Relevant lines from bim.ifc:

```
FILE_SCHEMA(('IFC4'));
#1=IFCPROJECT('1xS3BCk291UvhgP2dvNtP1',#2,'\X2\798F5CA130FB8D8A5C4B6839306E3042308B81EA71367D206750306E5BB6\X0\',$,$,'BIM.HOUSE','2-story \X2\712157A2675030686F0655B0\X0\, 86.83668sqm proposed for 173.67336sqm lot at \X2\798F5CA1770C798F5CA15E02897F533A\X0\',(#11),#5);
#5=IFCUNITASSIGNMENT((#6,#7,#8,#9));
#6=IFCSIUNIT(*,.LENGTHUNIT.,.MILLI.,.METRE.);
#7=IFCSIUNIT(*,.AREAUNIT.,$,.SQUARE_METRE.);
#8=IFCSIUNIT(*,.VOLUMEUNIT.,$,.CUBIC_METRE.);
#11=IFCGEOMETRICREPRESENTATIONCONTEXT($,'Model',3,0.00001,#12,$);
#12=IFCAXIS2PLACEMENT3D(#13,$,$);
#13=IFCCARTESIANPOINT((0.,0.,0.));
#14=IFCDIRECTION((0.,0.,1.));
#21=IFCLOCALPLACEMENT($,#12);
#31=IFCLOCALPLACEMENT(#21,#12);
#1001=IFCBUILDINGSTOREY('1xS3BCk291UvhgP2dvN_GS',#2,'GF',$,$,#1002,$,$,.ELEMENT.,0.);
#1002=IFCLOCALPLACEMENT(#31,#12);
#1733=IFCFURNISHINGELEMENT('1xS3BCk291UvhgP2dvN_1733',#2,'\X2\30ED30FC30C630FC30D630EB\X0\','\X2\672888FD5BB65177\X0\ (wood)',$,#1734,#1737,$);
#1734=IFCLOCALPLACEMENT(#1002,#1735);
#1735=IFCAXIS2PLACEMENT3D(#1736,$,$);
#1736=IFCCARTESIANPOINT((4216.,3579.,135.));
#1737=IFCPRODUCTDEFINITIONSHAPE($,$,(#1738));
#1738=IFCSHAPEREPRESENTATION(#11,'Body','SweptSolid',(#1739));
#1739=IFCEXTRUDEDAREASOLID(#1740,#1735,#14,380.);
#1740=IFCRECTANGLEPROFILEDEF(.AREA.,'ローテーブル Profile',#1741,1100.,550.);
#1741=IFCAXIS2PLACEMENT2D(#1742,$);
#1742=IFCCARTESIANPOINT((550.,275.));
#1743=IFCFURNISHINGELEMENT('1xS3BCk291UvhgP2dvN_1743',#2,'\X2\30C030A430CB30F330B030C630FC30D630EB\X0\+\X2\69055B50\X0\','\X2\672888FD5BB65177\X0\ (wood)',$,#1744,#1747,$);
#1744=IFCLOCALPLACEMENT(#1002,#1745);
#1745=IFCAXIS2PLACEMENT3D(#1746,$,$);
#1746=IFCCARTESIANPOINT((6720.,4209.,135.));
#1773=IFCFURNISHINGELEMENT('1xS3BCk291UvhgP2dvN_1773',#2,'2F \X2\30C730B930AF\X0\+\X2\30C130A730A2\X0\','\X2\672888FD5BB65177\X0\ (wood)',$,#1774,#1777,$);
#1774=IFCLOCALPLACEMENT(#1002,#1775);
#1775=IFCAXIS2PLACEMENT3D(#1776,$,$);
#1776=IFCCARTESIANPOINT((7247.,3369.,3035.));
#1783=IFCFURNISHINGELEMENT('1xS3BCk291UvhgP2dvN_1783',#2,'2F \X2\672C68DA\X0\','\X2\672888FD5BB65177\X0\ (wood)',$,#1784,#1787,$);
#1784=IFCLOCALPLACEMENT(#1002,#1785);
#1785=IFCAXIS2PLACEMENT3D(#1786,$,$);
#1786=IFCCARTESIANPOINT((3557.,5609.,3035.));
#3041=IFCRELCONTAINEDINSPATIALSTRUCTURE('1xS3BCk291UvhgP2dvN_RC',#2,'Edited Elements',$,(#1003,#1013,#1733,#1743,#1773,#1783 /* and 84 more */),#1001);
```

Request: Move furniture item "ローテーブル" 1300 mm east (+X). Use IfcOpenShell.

```python
import ifcopenshell
import ifcopenshell.api.geometry
import ifcopenshell.util.placement
import ifcopenshell.util.unit

model = ifcopenshell.open("bim.ifc")
unit_scale = ifcopenshell.util.unit.calculate_unit_scale(model)

item = model.by_guid("1xS3BCk291UvhgP2dvN_1733")
matrix = ifcopenshell.util.placement.get_local_placement(item.ObjectPlacement)
matrix[0, 3] += 1.3 / unit_scale
ifcopenshell.api.geometry.edit_object_placement(model, product=item, matrix=matrix, is_si=False)

print(ifcopenshell.util.placement.get_local_placement(item.ObjectPlacement).round(3) + 0.0)

model.write("bim_v2.ifc")
```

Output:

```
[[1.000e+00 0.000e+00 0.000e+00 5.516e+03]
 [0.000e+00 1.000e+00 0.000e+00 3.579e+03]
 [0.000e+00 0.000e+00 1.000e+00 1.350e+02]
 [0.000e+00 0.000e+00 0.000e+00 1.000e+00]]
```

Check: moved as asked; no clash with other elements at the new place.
